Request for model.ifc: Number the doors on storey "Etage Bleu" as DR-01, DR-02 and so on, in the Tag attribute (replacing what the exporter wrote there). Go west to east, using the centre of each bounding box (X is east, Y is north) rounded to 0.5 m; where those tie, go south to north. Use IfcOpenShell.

First a look at what the model holds.

```python
import ifcopenshell
import ifcopenshell.util.element
import ifcopenshell.util.placement

model = ifcopenshell.open("model.ifc")
print(model.schema)
storey = next(s for s in model.by_type("IfcBuildingStorey") if s.Name == "Etage Bleu")
doors = [e for e in ifcopenshell.util.element.get_decomposition(storey) if e.is_a("IfcDoor")]
for e in sorted(doors, key=lambda e: e.id()):
    origin = ifcopenshell.util.placement.get_local_placement(e.ObjectPlacement)[:3, 3]
    print(e.id(), e.Tag, e.Name, origin.round(2) + 0.0, sep=" | ")
```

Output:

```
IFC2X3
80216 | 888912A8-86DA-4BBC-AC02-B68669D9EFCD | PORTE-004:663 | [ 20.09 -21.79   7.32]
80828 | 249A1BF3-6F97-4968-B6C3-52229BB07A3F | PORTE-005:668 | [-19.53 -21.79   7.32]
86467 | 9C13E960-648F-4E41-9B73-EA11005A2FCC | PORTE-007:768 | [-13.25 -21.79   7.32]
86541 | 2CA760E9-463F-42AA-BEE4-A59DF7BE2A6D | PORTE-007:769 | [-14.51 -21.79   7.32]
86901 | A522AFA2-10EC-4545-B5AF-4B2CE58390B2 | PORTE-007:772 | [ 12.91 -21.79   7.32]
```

```python
import ifcopenshell
import ifcopenshell.geom
import ifcopenshell.util.element
import ifcopenshell.util.shape

model = ifcopenshell.open("model.ifc")
settings = ifcopenshell.geom.settings()
settings.set("use-world-coords", True)


def centre(element):
    shape = ifcopenshell.geom.create_shape(settings, element)
    return ifcopenshell.util.shape.get_bbox_centroid(shape.geometry)


storey = next(s for s in model.by_type("IfcBuildingStorey") if s.Name == "Etage Bleu")
doors = [e for e in ifcopenshell.util.element.get_decomposition(storey) if e.is_a("IfcDoor")]

# Insertion points can sit at a corner or the storey origin, so sort by the geometry (in metres).
centres = {e: centre(e) for e in doors}
doors.sort(key=lambda e: (round(centres[e][0] / 0.5), centres[e][1]))

for i, e in enumerate(doors, start=1):
    number = f"DR-{i:02d}"
    e.Tag = number
    print(e.id(), number)

model.write("model_updated.ifc")
```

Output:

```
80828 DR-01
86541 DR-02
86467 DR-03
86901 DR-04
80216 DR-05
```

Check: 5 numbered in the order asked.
